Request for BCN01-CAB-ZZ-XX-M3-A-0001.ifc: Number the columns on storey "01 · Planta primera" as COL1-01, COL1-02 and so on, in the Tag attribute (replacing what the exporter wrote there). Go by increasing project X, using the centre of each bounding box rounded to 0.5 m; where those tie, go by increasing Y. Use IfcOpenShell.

First a look at what the model holds.

```python
import ifcopenshell
import ifcopenshell.util.element
import ifcopenshell.util.placement

model = ifcopenshell.open("BCN01-CAB-ZZ-XX-M3-A-0001.ifc")
print(model.schema)
storey = next(s for s in model.by_type("IfcBuildingStorey") if s.Name == "01 · Planta primera")
columns = [e for e in ifcopenshell.util.element.get_decomposition(storey) if e.is_a("IfcColumn")]
for e in sorted(columns, key=lambda e: e.id()):
    origin = ifcopenshell.util.placement.get_local_placement(e.ObjectPlacement)[:3, 3]
    print(e.id(), e.Tag, e.Name, origin.round(2) + 0.0, sep=" | ")
```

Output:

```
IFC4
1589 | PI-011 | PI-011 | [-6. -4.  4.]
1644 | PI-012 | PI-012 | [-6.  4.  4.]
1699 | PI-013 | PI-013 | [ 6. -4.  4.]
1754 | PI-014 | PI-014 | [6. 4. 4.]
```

```python
import ifcopenshell
import ifcopenshell.geom
import ifcopenshell.util.element
import ifcopenshell.util.shape

model = ifcopenshell.open("BCN01-CAB-ZZ-XX-M3-A-0001.ifc")
settings = ifcopenshell.geom.settings()
settings.set("use-world-coords", True)


def centre(element):
    shape = ifcopenshell.geom.create_shape(settings, element)
    return ifcopenshell.util.shape.get_bbox_centroid(shape.geometry)


storey = next(s for s in model.by_type("IfcBuildingStorey") if s.Name == "01 · Planta primera")
columns = [e for e in ifcopenshell.util.element.get_decomposition(storey) if e.is_a("IfcColumn")]

# Insertion points can sit at a corner or the storey origin, so sort by the geometry (in metres).
centres = {e: centre(e) for e in columns}
columns.sort(key=lambda e: (round(centres[e][0] / 0.5), centres[e][1]))

for i, e in enumerate(columns, start=1):
    number = f"COL1-{i:02d}"
    e.Tag = number
    print(e.id(), number)

model.write("BCN01-CAB-ZZ-XX-M3-A-0001_v2.ifc")
```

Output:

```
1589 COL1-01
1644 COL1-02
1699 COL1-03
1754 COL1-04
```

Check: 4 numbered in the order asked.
